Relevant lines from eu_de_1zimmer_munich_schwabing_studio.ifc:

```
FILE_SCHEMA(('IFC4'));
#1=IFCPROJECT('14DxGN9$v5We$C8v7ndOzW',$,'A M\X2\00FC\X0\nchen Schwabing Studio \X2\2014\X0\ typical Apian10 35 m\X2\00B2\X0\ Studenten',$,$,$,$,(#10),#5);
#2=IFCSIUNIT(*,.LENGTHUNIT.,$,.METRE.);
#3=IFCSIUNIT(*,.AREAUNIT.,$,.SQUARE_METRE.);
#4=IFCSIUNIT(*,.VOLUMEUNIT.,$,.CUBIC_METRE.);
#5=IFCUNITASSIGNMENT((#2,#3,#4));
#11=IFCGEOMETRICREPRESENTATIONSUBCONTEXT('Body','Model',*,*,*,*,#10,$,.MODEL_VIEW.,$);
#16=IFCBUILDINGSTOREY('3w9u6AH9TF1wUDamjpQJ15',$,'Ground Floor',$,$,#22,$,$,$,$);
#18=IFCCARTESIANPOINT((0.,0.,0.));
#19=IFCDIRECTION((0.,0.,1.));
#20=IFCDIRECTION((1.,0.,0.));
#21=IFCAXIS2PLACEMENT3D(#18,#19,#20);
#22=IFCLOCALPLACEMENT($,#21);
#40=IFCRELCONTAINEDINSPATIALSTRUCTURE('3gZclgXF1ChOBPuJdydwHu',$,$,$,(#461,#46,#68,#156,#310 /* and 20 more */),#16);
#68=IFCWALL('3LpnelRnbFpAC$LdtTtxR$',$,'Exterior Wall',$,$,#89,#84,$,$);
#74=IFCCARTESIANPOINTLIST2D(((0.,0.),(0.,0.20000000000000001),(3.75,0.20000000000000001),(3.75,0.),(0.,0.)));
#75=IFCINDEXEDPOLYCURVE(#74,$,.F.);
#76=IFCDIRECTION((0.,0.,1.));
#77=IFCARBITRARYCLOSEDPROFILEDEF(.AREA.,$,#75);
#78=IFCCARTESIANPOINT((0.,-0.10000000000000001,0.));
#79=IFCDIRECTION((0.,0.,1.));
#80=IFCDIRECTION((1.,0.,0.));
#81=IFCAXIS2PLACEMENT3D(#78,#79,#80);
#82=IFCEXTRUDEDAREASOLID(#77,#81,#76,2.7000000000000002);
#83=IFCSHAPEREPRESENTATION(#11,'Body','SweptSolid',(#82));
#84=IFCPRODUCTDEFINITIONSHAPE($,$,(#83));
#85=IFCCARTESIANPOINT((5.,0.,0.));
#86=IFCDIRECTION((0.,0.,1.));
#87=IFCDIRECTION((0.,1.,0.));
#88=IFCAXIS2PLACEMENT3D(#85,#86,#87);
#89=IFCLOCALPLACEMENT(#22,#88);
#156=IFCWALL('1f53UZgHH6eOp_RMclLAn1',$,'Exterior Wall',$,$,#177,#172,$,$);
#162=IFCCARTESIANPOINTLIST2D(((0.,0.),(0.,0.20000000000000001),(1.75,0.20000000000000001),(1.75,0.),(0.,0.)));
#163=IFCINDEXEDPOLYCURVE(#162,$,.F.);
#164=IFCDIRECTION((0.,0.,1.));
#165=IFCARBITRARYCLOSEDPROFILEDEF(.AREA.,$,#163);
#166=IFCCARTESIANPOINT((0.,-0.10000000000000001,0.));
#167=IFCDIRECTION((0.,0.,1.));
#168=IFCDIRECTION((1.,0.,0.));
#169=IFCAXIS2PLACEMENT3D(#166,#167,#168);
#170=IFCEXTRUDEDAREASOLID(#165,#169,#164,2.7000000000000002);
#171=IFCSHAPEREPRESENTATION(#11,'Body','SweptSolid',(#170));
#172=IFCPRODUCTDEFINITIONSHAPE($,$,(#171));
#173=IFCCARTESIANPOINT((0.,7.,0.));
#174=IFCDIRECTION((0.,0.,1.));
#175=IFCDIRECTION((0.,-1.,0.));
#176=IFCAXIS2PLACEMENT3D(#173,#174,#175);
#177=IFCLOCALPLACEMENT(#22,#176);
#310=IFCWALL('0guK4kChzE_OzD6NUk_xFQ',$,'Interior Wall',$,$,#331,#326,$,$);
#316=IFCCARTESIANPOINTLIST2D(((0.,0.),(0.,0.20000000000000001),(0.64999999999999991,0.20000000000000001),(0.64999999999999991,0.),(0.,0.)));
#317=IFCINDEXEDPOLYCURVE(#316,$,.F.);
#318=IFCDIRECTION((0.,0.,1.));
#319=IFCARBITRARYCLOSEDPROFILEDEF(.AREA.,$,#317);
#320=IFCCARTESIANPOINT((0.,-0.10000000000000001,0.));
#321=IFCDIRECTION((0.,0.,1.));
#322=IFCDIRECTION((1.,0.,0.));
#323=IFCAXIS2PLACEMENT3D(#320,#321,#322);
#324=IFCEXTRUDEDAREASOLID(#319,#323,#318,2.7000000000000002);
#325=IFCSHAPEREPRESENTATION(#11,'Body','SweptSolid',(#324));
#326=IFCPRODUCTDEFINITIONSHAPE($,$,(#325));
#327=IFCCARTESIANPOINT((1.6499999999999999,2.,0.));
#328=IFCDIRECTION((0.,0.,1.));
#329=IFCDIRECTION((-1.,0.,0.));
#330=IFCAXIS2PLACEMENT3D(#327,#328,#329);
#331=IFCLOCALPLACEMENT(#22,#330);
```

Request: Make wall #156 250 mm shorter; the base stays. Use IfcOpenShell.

```python
import ifcopenshell
import ifcopenshell.geom
import ifcopenshell.util.representation
import ifcopenshell.util.shape

model = ifcopenshell.open("eu_de_1zimmer_munich_schwabing_studio.ifc")
settings = ifcopenshell.geom.settings()


def volume(element):
    """Net volume in cubic metres, openings subtracted."""
    shape = ifcopenshell.geom.create_shape(settings, element)
    return ifcopenshell.util.shape.get_volume(shape.geometry)


wall = model.by_guid("1f53UZgHH6eOp_RMclLAn1")
before = volume(wall)

body = ifcopenshell.util.representation.get_representation(wall, "Model", "Body")
solid = body.Items[0]
old_height = solid.Depth
solid.Depth -= 0.25
after = volume(wall)

print(f"height {old_height:g} -> {solid.Depth:g}, volume {before:.3f} -> {after:.3f} m3")

model.write("eu_de_1zimmer_munich_schwabing_studio_v2.ifc")
```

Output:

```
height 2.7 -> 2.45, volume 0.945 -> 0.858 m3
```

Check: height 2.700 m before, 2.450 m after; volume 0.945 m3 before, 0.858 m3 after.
